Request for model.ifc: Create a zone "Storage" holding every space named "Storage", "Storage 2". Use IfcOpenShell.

First a look at what the model holds.

```python
import ifcopenshell

model = ifcopenshell.open("model.ifc")
print(model.schema)
seen = {}
for space in model.by_type("IfcSpace"):
    seen[space.LongName] = seen.get(space.LongName, 0) + 1
for name, count in sorted(seen.items(), key=str):
    print(count, "x", name)
print("zones:", [z.Name for z in model.by_type("IfcZone")][:20])
```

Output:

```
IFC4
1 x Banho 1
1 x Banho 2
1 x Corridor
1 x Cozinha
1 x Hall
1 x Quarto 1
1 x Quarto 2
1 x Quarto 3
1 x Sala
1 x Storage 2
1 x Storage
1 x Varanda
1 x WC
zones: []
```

```python
import ifcopenshell
import ifcopenshell.api.group
import ifcopenshell.api.root

model = ifcopenshell.open("model.ifc")

names = {"Storage", "Storage 2"}
spaces = [s for s in model.by_type("IfcSpace") if s.LongName in names]

zone = ifcopenshell.api.root.create_entity(model, ifc_class="IfcZone", name="Storage")
ifcopenshell.api.group.assign_group(model, products=spaces, group=zone)
print(len(spaces), "spaces in", zone.Name)

model.write("model_v2.ifc")
```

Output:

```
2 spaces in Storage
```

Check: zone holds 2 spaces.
